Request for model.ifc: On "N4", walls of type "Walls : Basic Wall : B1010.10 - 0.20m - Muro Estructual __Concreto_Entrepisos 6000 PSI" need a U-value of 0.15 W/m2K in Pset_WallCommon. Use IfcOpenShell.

First a look at what the model holds.

```python
import ifcopenshell
import ifcopenshell.util.element

model = ifcopenshell.open("model.ifc")
print(model.schema)
storey = next(s for s in model.by_type("IfcBuildingStorey") if s.Name == "N4")
walls = [e for e in ifcopenshell.util.element.get_decomposition(storey) if e.is_a("IfcWall")]
seen = {}
for e in walls:
    element_type = ifcopenshell.util.element.get_type(e)
    key = (element_type.Name if element_type != e and element_type else None, ifcopenshell.util.element.get_pset(e, "Pset_WallCommon", "ThermalTransmittance"))
    seen[key] = seen.get(key, 0) + 1
for (name, value), count in sorted(seen.items(), key=str):
    print(count, "x", name, "|", value)
```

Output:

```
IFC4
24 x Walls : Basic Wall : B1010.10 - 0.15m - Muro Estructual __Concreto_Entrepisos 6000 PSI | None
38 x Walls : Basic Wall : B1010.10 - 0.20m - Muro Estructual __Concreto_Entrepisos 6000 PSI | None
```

```python
import ifcopenshell
import ifcopenshell.api.pset
import ifcopenshell.util.element

model = ifcopenshell.open("model.ifc")

storey = next(s for s in model.by_type("IfcBuildingStorey") if s.Name == "N4")
walls = [e for e in ifcopenshell.util.element.get_decomposition(storey) if e.is_a("IfcWall")]

count = 0
for e in walls:
    element_type = ifcopenshell.util.element.get_type(e)
    if element_type in (None, e) or element_type.Name != "Walls : Basic Wall : B1010.10 - 0.20m - Muro Estructual __Concreto_Entrepisos 6000 PSI":
        continue
    # add_pset returns the element's existing set when there is one.
    pset = ifcopenshell.api.pset.add_pset(model, product=e, name="Pset_WallCommon")
    ifcopenshell.api.pset.edit_pset(model, pset=pset, properties={"ThermalTransmittance": 0.15})
    count += 1

print(count, "walls updated")

model.write("model_edited.ifc")
```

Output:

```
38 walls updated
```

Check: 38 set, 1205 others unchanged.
